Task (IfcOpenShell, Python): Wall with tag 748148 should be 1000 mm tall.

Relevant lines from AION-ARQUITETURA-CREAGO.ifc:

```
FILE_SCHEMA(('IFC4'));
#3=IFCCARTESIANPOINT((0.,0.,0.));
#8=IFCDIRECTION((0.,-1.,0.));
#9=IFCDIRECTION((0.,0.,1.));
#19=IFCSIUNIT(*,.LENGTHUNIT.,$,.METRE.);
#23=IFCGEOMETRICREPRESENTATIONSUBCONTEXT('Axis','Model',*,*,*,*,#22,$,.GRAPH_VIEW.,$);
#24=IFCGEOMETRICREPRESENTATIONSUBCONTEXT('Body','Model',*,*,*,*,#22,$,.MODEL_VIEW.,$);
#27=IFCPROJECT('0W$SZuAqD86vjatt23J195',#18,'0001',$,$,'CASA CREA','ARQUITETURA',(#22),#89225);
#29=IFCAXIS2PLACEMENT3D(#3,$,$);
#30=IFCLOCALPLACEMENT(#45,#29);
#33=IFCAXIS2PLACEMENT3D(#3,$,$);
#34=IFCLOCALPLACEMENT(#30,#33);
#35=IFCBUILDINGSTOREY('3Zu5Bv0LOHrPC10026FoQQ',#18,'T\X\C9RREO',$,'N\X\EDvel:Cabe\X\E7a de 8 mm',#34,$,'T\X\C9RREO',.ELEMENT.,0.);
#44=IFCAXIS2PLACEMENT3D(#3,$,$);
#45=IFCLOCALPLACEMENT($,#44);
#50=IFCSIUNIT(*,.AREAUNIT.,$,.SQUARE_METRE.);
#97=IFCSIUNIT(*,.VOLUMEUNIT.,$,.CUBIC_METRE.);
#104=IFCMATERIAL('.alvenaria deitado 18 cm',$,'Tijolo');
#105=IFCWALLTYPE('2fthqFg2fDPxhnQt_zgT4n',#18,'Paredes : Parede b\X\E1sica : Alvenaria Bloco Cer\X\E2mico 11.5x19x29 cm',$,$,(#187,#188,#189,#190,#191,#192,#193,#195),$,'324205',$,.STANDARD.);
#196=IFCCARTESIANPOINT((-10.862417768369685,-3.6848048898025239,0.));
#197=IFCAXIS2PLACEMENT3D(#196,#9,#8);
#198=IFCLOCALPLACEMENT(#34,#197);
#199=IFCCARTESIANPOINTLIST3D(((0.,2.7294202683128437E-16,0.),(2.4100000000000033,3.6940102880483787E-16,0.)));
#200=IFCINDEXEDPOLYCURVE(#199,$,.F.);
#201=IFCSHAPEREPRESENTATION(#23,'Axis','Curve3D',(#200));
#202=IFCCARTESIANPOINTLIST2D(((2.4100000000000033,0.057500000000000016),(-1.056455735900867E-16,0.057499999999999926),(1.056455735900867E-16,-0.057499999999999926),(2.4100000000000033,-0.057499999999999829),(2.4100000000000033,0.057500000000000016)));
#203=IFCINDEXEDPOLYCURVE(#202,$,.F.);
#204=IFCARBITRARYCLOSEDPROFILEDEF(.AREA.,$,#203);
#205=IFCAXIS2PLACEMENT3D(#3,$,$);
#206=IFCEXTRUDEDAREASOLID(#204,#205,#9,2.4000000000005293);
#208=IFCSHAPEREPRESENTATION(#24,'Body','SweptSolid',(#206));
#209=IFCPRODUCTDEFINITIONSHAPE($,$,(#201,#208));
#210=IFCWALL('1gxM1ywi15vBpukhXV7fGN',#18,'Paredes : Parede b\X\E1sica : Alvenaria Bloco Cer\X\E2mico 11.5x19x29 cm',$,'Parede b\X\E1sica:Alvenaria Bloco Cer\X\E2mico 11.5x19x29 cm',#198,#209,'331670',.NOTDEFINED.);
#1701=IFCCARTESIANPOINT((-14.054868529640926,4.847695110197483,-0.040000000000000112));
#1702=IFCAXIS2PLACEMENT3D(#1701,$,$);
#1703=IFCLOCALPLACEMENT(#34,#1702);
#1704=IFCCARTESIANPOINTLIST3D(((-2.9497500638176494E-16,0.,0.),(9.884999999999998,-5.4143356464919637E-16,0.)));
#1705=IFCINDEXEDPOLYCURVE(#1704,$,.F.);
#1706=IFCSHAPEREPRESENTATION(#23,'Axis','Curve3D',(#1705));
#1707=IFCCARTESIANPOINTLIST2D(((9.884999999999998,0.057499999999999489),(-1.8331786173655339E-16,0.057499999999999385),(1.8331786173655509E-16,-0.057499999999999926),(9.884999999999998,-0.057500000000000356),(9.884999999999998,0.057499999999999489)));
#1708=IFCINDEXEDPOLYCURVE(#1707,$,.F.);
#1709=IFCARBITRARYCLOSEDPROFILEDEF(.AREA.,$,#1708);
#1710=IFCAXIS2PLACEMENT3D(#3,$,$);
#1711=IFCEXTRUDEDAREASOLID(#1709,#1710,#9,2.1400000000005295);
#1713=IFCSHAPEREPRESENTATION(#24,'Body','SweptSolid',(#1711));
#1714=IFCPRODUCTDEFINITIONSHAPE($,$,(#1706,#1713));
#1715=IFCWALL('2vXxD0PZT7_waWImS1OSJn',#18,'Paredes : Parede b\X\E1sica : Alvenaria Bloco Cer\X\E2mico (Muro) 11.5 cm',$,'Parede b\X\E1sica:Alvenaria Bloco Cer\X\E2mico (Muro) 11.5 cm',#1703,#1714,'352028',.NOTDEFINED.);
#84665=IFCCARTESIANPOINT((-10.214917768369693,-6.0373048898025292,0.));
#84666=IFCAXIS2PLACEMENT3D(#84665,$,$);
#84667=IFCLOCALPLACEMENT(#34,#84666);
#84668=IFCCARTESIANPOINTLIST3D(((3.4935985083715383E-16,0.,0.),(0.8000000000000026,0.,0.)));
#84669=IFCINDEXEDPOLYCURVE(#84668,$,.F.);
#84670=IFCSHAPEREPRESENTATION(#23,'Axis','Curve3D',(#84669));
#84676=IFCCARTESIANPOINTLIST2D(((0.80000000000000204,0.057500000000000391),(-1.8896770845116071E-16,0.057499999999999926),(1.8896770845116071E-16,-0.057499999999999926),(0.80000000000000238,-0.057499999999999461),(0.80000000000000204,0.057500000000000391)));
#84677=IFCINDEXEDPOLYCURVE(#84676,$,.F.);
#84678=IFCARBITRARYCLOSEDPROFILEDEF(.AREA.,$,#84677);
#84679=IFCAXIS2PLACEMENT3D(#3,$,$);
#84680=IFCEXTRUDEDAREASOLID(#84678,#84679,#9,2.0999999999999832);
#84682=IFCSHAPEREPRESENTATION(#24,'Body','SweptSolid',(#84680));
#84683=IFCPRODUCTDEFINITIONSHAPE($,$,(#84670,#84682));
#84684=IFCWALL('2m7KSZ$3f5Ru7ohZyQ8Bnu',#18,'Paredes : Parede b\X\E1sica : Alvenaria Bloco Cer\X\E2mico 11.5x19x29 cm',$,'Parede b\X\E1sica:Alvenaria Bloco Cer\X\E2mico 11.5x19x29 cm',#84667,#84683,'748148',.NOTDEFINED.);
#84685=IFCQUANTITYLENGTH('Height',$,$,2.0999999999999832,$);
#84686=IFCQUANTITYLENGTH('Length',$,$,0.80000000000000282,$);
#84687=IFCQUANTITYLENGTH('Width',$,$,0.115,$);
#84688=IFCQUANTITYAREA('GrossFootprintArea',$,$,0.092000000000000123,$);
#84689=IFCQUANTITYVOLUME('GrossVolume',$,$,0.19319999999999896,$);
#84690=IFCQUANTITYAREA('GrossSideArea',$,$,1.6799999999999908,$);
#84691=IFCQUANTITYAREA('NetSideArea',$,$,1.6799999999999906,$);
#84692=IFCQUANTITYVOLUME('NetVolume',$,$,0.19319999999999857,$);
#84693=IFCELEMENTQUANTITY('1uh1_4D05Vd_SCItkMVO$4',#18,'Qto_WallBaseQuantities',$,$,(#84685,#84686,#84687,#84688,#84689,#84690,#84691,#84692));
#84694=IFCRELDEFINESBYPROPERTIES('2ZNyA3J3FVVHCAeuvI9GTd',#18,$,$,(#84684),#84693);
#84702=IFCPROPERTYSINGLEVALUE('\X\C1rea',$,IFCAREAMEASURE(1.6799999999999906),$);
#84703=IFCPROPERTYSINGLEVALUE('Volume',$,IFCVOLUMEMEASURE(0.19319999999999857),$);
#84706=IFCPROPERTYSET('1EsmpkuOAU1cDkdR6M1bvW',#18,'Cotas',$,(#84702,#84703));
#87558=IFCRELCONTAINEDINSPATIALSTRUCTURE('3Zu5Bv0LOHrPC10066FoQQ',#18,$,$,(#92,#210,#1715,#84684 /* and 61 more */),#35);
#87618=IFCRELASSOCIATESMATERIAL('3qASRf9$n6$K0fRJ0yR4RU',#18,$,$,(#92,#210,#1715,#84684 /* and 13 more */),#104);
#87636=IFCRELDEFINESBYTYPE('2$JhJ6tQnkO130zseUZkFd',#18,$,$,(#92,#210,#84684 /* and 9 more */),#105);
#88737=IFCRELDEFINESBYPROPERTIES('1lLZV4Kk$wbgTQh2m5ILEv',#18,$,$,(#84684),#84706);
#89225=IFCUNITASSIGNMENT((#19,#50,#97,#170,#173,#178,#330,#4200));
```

```python
import ifcopenshell
import ifcopenshell.api.pset
import ifcopenshell.geom
import ifcopenshell.util.element
import ifcopenshell.util.representation
import ifcopenshell.util.shape
import ifcopenshell.util.unit

model = ifcopenshell.open("AION-ARQUITETURA-CREAGO.ifc")
unit_scale = ifcopenshell.util.unit.calculate_unit_scale(model)
area_scale = ifcopenshell.util.unit.calculate_unit_scale(model, "AREAUNIT")
volume_scale = ifcopenshell.util.unit.calculate_unit_scale(model, "VOLUMEUNIT")
settings = ifcopenshell.geom.settings()


def volume(element):
    """Net volume in cubic metres, openings subtracted."""
    shape = ifcopenshell.geom.create_shape(settings, element)
    return ifcopenshell.util.shape.get_volume(shape.geometry)


wall = model.by_guid("2m7KSZ$3f5Ru7ohZyQ8Bnu")
before = volume(wall)

body = ifcopenshell.util.representation.get_representation(wall, "Model", "Body")
solid = body.Items[0]
old_height = solid.Depth
solid.Depth = 1.0
after = volume(wall)
thickness = 0.115  # wall thickness in metres

# Update the stored height, areas and volumes.
qto = model.by_id(ifcopenshell.util.element.get_pset(wall, "Qto_WallBaseQuantities", should_inherit=False)["id"])
ifcopenshell.api.pset.edit_qto(model, qto=qto, properties={
    "Height": solid.Depth,
    "GrossVolume": ifcopenshell.util.element.get_pset(wall, "Qto_WallBaseQuantities", "GrossVolume") * solid.Depth / old_height,
    "GrossSideArea": ifcopenshell.util.element.get_pset(wall, "Qto_WallBaseQuantities", "GrossSideArea") * solid.Depth / old_height,
    "NetSideArea": after / thickness / area_scale,
    "NetVolume": after / volume_scale,
})
pset = model.by_id(ifcopenshell.util.element.get_pset(wall, "Cotas", should_inherit=False)["id"])
ifcopenshell.api.pset.edit_pset(model, pset=pset, properties={
    "Área": model.create_entity("IfcAreaMeasure", after / thickness / area_scale),
    "Volume": model.create_entity("IfcVolumeMeasure", after / volume_scale),
})

print(f"height {old_height:g} -> {solid.Depth:g}, volume {before:.3f} -> {after:.3f} m3")

model.write("AION-ARQUITETURA-CREAGO_edited.ifc")
```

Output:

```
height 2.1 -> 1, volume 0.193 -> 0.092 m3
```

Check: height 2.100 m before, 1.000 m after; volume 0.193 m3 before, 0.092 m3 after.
